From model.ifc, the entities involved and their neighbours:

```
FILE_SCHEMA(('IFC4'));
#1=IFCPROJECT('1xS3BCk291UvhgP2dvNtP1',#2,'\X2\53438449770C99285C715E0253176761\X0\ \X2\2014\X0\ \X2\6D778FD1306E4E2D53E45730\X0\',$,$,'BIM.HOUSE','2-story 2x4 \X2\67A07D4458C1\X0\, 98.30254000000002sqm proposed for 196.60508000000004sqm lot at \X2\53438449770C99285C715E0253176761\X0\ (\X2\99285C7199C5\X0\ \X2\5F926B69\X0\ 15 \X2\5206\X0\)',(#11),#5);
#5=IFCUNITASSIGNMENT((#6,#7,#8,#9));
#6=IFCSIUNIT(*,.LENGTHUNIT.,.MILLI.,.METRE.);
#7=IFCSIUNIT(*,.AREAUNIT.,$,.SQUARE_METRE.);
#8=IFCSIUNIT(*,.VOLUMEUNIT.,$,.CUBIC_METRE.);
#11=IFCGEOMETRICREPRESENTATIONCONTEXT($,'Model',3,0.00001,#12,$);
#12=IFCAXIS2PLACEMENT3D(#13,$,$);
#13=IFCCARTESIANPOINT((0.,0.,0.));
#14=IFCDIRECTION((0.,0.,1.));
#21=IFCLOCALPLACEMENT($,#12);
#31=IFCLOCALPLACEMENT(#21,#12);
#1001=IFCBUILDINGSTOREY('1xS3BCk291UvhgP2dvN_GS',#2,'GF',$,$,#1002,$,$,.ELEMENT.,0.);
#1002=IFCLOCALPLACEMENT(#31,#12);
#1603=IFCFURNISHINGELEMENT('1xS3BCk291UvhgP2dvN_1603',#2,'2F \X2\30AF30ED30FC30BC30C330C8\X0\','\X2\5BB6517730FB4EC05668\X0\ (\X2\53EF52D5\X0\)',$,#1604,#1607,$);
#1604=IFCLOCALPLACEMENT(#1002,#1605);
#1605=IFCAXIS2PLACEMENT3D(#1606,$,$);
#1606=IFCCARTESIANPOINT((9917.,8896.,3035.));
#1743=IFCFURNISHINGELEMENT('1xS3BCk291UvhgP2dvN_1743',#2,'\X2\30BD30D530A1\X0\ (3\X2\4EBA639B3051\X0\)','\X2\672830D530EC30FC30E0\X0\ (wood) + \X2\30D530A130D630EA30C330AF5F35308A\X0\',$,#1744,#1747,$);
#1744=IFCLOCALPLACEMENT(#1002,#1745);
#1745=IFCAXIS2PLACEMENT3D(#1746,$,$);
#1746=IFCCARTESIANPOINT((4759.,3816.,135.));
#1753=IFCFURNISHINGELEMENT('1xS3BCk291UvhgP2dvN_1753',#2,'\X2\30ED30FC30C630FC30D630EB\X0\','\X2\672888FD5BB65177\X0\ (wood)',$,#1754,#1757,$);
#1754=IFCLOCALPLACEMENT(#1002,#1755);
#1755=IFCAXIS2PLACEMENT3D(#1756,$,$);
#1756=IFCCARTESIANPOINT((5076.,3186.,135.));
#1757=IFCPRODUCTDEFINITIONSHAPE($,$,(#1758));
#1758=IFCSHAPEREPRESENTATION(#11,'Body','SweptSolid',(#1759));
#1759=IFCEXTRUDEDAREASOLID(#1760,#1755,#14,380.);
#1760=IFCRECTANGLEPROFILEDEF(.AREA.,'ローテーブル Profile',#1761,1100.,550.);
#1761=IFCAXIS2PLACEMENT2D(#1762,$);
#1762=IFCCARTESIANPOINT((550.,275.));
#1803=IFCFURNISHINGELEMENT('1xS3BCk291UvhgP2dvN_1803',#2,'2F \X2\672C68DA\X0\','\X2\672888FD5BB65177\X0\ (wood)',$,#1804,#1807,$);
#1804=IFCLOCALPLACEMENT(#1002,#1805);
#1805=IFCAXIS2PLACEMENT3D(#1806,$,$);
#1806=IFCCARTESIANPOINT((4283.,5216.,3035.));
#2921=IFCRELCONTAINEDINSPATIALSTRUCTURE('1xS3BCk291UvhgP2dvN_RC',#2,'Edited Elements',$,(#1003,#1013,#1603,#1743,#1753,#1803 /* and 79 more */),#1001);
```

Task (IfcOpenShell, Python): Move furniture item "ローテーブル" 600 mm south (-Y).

```python
import ifcopenshell
import ifcopenshell.api.geometry
import ifcopenshell.util.placement
import ifcopenshell.util.unit

model = ifcopenshell.open("model.ifc")
unit_scale = ifcopenshell.util.unit.calculate_unit_scale(model)

item = model.by_guid("1xS3BCk291UvhgP2dvN_1753")
matrix = ifcopenshell.util.placement.get_local_placement(item.ObjectPlacement)
matrix[1, 3] -= 0.6 / unit_scale
ifcopenshell.api.geometry.edit_object_placement(model, product=item, matrix=matrix, is_si=False)

print(ifcopenshell.util.placement.get_local_placement(item.ObjectPlacement).round(3) + 0.0)

model.write("model_edited.ifc")
```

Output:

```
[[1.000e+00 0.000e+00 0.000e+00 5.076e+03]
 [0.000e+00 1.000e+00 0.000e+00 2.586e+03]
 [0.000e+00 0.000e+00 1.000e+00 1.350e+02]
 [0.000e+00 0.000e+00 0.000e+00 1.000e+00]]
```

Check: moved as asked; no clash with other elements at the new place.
